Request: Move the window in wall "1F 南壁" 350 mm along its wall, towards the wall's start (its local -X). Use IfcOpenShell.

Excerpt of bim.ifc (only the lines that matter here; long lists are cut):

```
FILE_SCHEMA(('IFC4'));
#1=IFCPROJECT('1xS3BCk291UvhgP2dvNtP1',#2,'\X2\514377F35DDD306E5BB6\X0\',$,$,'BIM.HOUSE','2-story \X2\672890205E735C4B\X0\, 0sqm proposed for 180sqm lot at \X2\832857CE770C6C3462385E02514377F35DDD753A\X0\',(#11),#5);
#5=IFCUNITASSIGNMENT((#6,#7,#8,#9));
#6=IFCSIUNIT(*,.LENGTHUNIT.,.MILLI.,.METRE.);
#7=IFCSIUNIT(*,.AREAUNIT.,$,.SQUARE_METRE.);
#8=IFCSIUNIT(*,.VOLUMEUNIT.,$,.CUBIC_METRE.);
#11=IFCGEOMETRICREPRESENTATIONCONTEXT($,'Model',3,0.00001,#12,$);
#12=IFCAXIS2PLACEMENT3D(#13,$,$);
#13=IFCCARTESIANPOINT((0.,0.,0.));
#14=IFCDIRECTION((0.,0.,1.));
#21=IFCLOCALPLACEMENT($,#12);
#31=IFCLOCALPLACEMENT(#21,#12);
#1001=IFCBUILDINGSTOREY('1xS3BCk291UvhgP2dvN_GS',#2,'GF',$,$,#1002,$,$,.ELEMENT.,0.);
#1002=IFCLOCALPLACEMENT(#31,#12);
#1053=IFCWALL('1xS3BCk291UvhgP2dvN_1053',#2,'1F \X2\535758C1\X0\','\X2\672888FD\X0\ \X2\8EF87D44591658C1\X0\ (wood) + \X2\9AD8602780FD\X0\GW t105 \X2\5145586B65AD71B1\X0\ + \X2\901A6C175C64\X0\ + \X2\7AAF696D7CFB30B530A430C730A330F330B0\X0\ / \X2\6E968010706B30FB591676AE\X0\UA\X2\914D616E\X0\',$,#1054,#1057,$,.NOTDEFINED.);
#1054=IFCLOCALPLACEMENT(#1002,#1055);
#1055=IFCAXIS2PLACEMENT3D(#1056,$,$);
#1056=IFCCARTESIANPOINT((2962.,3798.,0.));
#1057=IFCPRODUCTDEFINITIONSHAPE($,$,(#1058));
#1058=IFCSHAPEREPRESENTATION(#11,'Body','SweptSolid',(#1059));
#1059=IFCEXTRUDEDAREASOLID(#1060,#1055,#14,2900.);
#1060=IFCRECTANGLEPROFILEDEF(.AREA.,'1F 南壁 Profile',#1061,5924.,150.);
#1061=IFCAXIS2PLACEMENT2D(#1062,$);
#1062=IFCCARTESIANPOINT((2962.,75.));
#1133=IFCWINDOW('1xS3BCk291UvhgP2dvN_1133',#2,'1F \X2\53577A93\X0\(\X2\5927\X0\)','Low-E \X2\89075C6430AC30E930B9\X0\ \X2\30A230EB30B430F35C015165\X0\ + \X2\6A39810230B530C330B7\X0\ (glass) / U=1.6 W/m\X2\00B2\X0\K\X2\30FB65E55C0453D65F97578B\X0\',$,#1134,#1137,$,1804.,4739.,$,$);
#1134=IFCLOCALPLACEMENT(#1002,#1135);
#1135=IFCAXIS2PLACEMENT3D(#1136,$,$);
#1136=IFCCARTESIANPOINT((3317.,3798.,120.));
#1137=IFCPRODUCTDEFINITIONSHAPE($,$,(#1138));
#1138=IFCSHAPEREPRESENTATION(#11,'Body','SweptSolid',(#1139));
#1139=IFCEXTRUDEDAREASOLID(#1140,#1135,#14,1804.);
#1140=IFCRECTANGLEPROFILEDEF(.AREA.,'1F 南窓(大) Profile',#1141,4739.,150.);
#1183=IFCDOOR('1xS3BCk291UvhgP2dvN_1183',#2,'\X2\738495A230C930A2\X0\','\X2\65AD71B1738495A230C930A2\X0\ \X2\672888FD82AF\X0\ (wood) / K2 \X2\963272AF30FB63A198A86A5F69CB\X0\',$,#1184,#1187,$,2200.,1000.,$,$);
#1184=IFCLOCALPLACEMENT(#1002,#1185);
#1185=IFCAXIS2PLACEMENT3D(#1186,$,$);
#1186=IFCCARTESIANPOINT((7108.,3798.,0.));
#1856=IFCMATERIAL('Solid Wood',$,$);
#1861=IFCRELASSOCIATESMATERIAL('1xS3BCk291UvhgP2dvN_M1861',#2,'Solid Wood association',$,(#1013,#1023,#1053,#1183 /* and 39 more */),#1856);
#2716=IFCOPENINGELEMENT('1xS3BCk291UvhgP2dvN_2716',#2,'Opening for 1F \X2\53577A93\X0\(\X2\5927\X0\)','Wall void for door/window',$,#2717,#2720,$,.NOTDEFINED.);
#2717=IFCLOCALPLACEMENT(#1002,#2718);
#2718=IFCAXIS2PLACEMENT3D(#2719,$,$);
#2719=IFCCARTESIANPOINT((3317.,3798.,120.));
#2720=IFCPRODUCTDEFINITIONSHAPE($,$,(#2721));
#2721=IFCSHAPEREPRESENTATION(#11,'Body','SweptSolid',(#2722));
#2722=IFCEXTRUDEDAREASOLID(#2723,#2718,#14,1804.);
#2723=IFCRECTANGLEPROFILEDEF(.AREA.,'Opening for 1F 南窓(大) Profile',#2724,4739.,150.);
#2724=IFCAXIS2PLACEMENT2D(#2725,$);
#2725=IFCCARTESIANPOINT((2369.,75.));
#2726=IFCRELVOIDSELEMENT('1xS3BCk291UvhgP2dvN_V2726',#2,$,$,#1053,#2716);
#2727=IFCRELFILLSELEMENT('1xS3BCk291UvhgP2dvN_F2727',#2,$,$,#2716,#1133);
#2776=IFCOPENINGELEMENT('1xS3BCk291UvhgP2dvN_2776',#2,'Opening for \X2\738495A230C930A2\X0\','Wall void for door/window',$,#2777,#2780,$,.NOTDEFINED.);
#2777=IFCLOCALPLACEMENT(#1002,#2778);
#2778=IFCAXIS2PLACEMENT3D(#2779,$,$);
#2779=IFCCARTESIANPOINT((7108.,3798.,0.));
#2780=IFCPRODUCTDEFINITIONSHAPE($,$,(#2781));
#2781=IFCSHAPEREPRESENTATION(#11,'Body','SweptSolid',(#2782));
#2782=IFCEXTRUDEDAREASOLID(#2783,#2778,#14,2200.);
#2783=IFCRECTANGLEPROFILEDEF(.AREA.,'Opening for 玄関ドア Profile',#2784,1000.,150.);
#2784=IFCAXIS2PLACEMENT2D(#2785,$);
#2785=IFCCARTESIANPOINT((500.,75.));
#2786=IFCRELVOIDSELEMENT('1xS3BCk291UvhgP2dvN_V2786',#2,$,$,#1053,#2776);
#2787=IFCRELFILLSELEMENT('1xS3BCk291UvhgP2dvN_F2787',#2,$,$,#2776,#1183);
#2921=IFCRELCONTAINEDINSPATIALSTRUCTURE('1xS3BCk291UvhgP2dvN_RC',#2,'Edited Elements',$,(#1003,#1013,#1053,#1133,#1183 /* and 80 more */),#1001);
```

```python
import ifcopenshell
import ifcopenshell.api.geometry
import ifcopenshell.util.placement
import ifcopenshell.util.unit

model = ifcopenshell.open("bim.ifc")
unit_scale = ifcopenshell.util.unit.calculate_unit_scale(model)

window = model.by_guid("1xS3BCk291UvhgP2dvN_1133")
opening = window.FillsVoids[0].RelatingOpeningElement
wall = opening.VoidsElements[0].RelatingBuildingElement

wall_matrix = ifcopenshell.util.placement.get_local_placement(wall.ObjectPlacement)
shift = wall_matrix[:3, 0] * -0.35 / unit_scale
before = ifcopenshell.util.placement.get_local_placement(window.ObjectPlacement)[:3, 3].copy()

# The window is not placed relative to its opening, so move both.
for product in (opening, window):
    matrix = ifcopenshell.util.placement.get_local_placement(product.ObjectPlacement)
    matrix[:3, 3] += shift
    ifcopenshell.api.geometry.edit_object_placement(model, product=product, matrix=matrix, is_si=False)

after = ifcopenshell.util.placement.get_local_placement(window.ObjectPlacement)[:3, 3]
print("window moved by", (after - before).round(3) + 0.0)

model.write("bim_edited.ifc")
```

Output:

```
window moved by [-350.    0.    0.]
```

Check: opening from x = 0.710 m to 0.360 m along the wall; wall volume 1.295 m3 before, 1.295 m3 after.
